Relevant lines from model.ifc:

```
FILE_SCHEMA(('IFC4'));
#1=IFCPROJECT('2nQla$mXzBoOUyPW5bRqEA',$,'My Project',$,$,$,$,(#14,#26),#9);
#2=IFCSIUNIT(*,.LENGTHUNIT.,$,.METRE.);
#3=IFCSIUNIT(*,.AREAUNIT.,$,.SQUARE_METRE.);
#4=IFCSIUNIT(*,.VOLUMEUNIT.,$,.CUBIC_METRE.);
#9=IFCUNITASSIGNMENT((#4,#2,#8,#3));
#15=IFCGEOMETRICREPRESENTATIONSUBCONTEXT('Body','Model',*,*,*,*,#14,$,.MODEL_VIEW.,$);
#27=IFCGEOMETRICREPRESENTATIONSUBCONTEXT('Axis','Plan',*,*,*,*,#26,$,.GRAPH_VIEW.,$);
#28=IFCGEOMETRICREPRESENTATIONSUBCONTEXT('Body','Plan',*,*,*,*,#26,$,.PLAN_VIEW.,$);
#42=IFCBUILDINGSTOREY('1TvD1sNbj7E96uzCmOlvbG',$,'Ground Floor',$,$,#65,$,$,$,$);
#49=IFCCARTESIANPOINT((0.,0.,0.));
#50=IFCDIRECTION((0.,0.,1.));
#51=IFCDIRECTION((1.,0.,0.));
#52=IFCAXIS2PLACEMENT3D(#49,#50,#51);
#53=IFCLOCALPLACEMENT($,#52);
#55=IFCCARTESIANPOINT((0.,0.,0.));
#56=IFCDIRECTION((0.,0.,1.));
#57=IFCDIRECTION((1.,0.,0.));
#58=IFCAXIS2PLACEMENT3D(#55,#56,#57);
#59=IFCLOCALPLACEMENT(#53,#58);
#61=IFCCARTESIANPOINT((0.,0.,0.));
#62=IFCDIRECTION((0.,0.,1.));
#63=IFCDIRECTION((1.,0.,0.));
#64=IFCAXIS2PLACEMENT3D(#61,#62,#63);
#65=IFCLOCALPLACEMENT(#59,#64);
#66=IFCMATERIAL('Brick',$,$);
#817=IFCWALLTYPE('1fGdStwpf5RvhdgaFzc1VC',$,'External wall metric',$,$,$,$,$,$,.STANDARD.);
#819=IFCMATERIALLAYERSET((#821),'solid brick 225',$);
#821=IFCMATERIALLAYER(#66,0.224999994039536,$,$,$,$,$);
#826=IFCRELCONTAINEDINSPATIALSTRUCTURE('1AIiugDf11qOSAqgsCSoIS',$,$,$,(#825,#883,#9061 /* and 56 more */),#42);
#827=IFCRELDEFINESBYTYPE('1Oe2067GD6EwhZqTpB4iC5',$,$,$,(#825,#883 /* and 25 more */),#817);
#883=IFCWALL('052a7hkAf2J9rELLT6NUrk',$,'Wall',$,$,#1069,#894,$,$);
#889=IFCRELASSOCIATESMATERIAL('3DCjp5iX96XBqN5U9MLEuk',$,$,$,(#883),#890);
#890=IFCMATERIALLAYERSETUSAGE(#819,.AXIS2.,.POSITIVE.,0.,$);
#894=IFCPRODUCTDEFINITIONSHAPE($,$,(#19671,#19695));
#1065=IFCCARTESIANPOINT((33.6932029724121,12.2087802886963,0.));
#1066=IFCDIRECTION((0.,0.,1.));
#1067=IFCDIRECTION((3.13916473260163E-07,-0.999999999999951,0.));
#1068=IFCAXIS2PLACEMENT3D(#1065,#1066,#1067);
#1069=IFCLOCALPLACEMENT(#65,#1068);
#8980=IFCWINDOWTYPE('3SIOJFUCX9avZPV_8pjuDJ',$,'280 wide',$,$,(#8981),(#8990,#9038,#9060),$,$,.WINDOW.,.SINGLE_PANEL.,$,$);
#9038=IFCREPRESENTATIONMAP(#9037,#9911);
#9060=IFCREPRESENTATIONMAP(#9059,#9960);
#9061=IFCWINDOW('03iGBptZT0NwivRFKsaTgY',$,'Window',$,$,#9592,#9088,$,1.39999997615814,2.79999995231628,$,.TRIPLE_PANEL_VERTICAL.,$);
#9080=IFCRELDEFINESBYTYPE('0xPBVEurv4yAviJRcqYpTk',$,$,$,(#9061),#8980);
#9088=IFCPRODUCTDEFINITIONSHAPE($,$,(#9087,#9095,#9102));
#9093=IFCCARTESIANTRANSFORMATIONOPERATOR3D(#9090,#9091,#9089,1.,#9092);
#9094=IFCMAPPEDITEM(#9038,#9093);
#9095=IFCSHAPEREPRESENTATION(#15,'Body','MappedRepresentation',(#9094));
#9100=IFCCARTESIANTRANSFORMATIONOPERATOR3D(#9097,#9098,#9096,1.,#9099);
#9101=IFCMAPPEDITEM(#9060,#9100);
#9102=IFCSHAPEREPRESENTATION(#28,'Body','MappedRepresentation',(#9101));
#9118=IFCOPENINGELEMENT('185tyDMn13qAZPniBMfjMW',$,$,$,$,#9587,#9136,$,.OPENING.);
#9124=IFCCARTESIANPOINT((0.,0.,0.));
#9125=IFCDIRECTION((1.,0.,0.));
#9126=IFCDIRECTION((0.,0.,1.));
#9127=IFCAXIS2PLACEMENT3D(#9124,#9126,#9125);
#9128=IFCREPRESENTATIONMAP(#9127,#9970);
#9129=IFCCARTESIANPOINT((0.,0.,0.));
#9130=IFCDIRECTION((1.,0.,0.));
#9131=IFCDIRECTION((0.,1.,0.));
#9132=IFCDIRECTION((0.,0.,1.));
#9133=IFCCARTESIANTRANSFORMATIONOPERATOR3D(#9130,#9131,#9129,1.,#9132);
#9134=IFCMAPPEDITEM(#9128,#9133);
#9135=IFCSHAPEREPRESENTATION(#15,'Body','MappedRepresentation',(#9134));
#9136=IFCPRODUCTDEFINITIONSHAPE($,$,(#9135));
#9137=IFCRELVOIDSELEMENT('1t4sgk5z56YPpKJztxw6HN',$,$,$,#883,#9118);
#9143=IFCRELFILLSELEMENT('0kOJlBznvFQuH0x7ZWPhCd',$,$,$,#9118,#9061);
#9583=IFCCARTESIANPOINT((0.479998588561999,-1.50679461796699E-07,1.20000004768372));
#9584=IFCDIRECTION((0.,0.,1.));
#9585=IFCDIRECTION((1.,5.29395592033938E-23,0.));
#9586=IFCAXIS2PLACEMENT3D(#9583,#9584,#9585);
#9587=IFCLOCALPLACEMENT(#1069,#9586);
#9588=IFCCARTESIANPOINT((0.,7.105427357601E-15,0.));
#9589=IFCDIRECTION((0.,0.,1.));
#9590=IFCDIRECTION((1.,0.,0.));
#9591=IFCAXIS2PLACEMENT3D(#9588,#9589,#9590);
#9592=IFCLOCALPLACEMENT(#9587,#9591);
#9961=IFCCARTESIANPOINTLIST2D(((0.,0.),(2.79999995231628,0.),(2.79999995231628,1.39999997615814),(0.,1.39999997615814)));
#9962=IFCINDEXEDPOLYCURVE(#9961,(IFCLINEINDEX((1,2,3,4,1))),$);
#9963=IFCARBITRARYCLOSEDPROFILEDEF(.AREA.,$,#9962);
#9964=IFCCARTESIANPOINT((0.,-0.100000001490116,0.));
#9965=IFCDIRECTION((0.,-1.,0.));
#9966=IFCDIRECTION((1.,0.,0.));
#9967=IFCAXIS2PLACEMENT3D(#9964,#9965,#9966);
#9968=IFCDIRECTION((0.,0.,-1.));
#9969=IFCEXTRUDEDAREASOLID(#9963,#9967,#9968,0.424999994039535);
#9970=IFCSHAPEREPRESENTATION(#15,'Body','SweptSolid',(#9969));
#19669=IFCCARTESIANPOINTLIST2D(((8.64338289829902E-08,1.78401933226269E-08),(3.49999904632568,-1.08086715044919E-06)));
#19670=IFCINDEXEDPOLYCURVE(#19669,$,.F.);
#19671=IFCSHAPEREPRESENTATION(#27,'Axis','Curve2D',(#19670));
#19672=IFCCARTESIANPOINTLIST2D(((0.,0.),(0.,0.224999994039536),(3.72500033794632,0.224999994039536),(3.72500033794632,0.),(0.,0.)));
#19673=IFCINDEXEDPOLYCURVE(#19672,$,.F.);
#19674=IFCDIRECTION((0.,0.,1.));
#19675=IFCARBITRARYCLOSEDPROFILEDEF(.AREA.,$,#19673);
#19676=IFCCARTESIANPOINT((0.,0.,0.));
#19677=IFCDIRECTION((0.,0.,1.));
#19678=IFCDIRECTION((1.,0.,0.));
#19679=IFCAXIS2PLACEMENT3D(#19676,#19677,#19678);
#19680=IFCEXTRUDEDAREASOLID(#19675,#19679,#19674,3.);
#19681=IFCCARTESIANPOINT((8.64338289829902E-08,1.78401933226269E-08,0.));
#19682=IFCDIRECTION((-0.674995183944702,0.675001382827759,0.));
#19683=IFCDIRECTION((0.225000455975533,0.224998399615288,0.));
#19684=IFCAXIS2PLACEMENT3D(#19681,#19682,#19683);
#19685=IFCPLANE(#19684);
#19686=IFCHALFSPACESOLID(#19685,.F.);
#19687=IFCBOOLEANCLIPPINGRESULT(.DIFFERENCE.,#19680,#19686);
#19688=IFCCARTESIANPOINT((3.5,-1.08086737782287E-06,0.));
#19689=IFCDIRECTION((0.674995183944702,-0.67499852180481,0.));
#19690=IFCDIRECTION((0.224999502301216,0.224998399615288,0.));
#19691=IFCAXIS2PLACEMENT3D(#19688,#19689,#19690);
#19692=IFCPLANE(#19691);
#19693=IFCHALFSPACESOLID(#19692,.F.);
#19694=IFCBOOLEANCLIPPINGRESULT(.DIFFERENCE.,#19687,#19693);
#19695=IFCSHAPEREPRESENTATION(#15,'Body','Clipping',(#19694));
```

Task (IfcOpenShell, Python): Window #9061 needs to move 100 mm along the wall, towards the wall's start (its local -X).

```python
import ifcopenshell
import ifcopenshell.api.geometry
import ifcopenshell.util.placement
import ifcopenshell.util.unit

model = ifcopenshell.open("model.ifc")
unit_scale = ifcopenshell.util.unit.calculate_unit_scale(model)

window = model.by_guid("03iGBptZT0NwivRFKsaTgY")
opening = window.FillsVoids[0].RelatingOpeningElement
wall = opening.VoidsElements[0].RelatingBuildingElement

wall_matrix = ifcopenshell.util.placement.get_local_placement(wall.ObjectPlacement)
shift = wall_matrix[:3, 0] * -0.1 / unit_scale
before = ifcopenshell.util.placement.get_local_placement(window.ObjectPlacement)[:3, 3].copy()

# The window is placed relative to its opening, so it follows when the opening moves.
matrix = ifcopenshell.util.placement.get_local_placement(opening.ObjectPlacement)
matrix[:3, 3] += shift
ifcopenshell.api.geometry.edit_object_placement(
    model, product=opening, matrix=matrix, is_si=False, should_transform_children=True
)

after = ifcopenshell.util.placement.get_local_placement(window.ObjectPlacement)[:3, 3]
print("window moved by", (after - before).round(3) + 0.0)

model.write("model_updated.ifc")
```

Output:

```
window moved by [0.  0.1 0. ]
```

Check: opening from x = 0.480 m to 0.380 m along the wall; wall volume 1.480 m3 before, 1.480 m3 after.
